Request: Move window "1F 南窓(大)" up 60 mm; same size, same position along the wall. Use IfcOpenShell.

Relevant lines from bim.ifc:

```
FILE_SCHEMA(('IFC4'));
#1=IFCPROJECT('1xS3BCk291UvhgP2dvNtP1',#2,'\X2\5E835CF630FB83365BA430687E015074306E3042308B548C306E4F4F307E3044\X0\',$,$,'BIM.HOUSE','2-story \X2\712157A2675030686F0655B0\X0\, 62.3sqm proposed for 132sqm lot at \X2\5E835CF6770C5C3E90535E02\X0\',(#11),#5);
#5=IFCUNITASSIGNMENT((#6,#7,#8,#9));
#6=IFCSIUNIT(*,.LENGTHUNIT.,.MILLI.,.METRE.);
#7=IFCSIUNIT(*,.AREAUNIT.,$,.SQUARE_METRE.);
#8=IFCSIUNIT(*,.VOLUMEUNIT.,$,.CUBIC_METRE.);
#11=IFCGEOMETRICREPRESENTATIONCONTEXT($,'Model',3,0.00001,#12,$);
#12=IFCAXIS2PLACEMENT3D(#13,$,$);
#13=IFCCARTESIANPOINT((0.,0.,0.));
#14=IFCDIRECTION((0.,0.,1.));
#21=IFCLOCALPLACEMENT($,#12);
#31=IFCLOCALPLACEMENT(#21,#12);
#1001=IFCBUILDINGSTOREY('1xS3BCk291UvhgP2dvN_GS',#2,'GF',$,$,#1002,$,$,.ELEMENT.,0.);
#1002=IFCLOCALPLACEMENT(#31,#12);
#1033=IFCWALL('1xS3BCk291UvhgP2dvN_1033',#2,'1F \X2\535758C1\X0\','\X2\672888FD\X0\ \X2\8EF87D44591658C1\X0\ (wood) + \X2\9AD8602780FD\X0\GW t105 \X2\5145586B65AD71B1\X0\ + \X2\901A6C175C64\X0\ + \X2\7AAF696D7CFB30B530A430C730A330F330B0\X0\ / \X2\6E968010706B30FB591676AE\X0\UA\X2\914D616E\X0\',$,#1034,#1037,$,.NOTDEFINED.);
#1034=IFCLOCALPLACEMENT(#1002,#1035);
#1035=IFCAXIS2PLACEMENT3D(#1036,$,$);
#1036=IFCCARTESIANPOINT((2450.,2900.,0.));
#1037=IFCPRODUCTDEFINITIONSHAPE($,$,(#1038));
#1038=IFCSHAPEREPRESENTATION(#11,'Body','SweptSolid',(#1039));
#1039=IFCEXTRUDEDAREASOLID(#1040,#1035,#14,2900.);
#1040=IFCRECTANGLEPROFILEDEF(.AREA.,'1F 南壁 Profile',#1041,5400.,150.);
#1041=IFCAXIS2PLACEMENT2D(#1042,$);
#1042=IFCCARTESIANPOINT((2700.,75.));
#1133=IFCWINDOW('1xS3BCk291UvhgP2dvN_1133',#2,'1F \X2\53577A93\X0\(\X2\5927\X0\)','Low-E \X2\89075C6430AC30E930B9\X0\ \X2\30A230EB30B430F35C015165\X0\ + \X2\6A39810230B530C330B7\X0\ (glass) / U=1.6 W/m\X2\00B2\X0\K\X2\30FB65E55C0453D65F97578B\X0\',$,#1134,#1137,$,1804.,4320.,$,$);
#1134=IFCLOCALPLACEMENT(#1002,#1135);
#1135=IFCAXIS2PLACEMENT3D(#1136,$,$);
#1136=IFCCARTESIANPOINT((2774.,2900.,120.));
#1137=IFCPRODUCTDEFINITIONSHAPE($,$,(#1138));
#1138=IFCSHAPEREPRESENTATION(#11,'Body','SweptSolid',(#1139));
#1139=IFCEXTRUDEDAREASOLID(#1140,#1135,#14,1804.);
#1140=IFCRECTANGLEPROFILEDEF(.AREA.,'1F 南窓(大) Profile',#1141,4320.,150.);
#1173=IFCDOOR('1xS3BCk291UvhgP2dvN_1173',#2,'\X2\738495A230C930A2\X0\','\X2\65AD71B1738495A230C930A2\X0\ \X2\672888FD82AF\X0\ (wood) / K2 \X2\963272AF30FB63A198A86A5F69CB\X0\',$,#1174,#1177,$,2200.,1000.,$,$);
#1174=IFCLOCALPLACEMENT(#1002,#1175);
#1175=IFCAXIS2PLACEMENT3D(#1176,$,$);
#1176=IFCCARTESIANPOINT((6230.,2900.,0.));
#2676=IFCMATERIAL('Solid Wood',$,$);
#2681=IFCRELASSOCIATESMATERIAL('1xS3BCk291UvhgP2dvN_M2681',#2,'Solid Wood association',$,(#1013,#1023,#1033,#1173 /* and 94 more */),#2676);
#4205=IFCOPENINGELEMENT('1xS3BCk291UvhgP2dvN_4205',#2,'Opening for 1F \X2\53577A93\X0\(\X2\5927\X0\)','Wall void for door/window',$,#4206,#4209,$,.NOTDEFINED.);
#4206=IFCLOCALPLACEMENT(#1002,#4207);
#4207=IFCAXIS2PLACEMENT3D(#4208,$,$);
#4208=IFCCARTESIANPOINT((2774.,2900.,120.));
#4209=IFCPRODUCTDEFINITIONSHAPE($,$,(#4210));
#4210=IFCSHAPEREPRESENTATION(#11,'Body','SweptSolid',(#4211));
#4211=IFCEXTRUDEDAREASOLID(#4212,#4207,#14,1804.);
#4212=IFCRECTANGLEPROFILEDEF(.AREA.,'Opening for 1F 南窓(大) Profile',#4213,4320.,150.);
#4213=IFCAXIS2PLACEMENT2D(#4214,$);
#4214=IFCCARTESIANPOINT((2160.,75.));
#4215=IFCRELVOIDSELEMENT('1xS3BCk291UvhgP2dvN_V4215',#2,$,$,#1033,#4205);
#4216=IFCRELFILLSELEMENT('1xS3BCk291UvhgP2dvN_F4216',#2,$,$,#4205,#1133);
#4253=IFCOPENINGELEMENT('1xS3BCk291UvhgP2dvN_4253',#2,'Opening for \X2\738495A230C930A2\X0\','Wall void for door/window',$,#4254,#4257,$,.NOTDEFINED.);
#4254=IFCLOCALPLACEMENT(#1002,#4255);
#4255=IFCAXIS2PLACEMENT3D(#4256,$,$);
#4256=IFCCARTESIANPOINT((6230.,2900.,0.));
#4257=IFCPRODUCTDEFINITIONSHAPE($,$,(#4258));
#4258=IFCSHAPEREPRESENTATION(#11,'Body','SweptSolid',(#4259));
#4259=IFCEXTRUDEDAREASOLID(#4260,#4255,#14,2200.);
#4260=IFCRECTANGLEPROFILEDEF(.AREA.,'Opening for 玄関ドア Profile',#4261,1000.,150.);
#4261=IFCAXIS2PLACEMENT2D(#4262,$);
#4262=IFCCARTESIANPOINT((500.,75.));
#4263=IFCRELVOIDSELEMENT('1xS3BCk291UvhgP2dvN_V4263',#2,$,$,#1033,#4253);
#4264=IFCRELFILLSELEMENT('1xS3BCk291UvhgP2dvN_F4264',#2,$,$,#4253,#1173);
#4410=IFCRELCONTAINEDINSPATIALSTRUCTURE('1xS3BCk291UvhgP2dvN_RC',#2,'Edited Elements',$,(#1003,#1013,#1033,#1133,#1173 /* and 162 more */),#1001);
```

```python
import numpy as np
import ifcopenshell
import ifcopenshell.api.geometry
import ifcopenshell.util.placement
import ifcopenshell.util.unit

model = ifcopenshell.open("bim.ifc")
unit_scale = ifcopenshell.util.unit.calculate_unit_scale(model)

window = model.by_guid("1xS3BCk291UvhgP2dvN_1133")
opening = window.FillsVoids[0].RelatingOpeningElement
dz = 0.06 / unit_scale

shift = np.array([0.0, 0.0, dz])
# The window is not placed relative to its opening, so move both.
for product in (opening, window):
    matrix = ifcopenshell.util.placement.get_local_placement(product.ObjectPlacement)
    matrix[:3, 3] += shift
    ifcopenshell.api.geometry.edit_object_placement(model, product=product, matrix=matrix, is_si=False)

print(f"moved by {dz * unit_scale:+.3f} m")

model.write("bim_updated.ifc")
```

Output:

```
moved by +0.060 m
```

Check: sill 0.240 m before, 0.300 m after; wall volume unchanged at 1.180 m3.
